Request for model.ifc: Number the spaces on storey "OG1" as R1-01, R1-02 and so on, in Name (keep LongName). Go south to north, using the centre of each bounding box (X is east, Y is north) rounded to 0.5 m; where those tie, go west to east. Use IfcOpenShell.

First a look at what the model holds.

```python
import ifcopenshell
import ifcopenshell.util.element
import ifcopenshell.util.placement

model = ifcopenshell.open("model.ifc")
print(model.schema)
storey = next(s for s in model.by_type("IfcBuildingStorey") if s.Name == "OG1")
spaces = [e for e in ifcopenshell.util.element.get_decomposition(storey) if e.is_a("IfcSpace")]
for e in sorted(spaces, key=lambda e: e.id()):
    origin = ifcopenshell.util.placement.get_local_placement(e.ObjectPlacement)[:3, 3]
    print(e.id(), e.Name, e.LongName, origin.round(2) + 0.0, sep=" | ")
```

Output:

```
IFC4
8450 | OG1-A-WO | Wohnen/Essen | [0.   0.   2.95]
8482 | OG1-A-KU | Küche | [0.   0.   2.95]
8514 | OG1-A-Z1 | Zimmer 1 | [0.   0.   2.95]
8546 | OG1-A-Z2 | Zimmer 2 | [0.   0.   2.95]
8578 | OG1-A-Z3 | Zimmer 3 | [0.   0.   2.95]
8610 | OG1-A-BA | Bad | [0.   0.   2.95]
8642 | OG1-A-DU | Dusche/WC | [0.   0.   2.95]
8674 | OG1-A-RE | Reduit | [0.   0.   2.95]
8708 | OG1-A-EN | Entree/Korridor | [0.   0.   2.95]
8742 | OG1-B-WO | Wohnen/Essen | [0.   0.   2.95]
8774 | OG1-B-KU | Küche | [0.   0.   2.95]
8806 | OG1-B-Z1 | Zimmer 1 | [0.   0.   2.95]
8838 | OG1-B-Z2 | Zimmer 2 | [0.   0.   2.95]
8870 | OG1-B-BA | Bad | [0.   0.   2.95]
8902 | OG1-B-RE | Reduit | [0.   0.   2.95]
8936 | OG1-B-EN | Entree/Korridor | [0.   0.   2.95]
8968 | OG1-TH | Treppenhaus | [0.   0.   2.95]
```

```python
import ifcopenshell
import ifcopenshell.geom
import ifcopenshell.util.element
import ifcopenshell.util.shape

model = ifcopenshell.open("model.ifc")
settings = ifcopenshell.geom.settings()
settings.set("use-world-coords", True)


def centre(element):
    shape = ifcopenshell.geom.create_shape(settings, element)
    return ifcopenshell.util.shape.get_bbox_centroid(shape.geometry)


storey = next(s for s in model.by_type("IfcBuildingStorey") if s.Name == "OG1")
spaces = [e for e in ifcopenshell.util.element.get_decomposition(storey) if e.is_a("IfcSpace")]

# Insertion points can sit at a corner or the storey origin, so sort by the geometry (in metres).
centres = {e: centre(e) for e in spaces}
spaces.sort(key=lambda e: (round(centres[e][1] / 0.5), centres[e][0]))

for i, e in enumerate(spaces, start=1):
    number = f"R1-{i:02d}"
    e.Name = number
    print(e.id(), number)

model.write("model_v2.ifc")
```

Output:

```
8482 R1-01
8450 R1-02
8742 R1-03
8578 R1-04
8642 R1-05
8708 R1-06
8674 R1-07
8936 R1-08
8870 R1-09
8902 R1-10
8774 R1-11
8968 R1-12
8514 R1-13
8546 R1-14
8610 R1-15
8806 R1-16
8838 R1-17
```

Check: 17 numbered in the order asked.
